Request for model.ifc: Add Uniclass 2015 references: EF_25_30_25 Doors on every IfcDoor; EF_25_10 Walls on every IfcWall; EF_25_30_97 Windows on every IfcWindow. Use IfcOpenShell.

First a look at what the model holds.

```python
import ifcopenshell

model = ifcopenshell.open("model.ifc")
print(model.schema)
print("classifications:", [c.Name for c in model.by_type("IfcClassification")])
for ifc_class in ("IfcDoor", "IfcRoof", "IfcStair", "IfcWall", "IfcWindow"):
    print(ifc_class, len(model.by_type(ifc_class)))
```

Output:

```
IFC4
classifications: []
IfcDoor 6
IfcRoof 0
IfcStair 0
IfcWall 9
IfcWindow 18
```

```python
import ifcopenshell
import ifcopenshell.api.classification

model = ifcopenshell.open("model.ifc")

system = ifcopenshell.api.classification.add_classification(model, classification="Uniclass 2015")

codes = {
    "IfcDoor": ("EF_25_30_25", "Doors"),
    "IfcWall": ("EF_25_10", "Walls"),
    "IfcWindow": ("EF_25_30_97", "Windows"),
}
for ifc_class, (code, name) in codes.items():
    products = model.by_type(ifc_class)
    ifcopenshell.api.classification.add_reference(
        model, products=products, classification=system, identification=code, name=name
    )
    print(code, len(products))

model.write("model_v2.ifc")
```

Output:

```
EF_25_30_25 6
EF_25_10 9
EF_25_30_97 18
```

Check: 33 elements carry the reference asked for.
